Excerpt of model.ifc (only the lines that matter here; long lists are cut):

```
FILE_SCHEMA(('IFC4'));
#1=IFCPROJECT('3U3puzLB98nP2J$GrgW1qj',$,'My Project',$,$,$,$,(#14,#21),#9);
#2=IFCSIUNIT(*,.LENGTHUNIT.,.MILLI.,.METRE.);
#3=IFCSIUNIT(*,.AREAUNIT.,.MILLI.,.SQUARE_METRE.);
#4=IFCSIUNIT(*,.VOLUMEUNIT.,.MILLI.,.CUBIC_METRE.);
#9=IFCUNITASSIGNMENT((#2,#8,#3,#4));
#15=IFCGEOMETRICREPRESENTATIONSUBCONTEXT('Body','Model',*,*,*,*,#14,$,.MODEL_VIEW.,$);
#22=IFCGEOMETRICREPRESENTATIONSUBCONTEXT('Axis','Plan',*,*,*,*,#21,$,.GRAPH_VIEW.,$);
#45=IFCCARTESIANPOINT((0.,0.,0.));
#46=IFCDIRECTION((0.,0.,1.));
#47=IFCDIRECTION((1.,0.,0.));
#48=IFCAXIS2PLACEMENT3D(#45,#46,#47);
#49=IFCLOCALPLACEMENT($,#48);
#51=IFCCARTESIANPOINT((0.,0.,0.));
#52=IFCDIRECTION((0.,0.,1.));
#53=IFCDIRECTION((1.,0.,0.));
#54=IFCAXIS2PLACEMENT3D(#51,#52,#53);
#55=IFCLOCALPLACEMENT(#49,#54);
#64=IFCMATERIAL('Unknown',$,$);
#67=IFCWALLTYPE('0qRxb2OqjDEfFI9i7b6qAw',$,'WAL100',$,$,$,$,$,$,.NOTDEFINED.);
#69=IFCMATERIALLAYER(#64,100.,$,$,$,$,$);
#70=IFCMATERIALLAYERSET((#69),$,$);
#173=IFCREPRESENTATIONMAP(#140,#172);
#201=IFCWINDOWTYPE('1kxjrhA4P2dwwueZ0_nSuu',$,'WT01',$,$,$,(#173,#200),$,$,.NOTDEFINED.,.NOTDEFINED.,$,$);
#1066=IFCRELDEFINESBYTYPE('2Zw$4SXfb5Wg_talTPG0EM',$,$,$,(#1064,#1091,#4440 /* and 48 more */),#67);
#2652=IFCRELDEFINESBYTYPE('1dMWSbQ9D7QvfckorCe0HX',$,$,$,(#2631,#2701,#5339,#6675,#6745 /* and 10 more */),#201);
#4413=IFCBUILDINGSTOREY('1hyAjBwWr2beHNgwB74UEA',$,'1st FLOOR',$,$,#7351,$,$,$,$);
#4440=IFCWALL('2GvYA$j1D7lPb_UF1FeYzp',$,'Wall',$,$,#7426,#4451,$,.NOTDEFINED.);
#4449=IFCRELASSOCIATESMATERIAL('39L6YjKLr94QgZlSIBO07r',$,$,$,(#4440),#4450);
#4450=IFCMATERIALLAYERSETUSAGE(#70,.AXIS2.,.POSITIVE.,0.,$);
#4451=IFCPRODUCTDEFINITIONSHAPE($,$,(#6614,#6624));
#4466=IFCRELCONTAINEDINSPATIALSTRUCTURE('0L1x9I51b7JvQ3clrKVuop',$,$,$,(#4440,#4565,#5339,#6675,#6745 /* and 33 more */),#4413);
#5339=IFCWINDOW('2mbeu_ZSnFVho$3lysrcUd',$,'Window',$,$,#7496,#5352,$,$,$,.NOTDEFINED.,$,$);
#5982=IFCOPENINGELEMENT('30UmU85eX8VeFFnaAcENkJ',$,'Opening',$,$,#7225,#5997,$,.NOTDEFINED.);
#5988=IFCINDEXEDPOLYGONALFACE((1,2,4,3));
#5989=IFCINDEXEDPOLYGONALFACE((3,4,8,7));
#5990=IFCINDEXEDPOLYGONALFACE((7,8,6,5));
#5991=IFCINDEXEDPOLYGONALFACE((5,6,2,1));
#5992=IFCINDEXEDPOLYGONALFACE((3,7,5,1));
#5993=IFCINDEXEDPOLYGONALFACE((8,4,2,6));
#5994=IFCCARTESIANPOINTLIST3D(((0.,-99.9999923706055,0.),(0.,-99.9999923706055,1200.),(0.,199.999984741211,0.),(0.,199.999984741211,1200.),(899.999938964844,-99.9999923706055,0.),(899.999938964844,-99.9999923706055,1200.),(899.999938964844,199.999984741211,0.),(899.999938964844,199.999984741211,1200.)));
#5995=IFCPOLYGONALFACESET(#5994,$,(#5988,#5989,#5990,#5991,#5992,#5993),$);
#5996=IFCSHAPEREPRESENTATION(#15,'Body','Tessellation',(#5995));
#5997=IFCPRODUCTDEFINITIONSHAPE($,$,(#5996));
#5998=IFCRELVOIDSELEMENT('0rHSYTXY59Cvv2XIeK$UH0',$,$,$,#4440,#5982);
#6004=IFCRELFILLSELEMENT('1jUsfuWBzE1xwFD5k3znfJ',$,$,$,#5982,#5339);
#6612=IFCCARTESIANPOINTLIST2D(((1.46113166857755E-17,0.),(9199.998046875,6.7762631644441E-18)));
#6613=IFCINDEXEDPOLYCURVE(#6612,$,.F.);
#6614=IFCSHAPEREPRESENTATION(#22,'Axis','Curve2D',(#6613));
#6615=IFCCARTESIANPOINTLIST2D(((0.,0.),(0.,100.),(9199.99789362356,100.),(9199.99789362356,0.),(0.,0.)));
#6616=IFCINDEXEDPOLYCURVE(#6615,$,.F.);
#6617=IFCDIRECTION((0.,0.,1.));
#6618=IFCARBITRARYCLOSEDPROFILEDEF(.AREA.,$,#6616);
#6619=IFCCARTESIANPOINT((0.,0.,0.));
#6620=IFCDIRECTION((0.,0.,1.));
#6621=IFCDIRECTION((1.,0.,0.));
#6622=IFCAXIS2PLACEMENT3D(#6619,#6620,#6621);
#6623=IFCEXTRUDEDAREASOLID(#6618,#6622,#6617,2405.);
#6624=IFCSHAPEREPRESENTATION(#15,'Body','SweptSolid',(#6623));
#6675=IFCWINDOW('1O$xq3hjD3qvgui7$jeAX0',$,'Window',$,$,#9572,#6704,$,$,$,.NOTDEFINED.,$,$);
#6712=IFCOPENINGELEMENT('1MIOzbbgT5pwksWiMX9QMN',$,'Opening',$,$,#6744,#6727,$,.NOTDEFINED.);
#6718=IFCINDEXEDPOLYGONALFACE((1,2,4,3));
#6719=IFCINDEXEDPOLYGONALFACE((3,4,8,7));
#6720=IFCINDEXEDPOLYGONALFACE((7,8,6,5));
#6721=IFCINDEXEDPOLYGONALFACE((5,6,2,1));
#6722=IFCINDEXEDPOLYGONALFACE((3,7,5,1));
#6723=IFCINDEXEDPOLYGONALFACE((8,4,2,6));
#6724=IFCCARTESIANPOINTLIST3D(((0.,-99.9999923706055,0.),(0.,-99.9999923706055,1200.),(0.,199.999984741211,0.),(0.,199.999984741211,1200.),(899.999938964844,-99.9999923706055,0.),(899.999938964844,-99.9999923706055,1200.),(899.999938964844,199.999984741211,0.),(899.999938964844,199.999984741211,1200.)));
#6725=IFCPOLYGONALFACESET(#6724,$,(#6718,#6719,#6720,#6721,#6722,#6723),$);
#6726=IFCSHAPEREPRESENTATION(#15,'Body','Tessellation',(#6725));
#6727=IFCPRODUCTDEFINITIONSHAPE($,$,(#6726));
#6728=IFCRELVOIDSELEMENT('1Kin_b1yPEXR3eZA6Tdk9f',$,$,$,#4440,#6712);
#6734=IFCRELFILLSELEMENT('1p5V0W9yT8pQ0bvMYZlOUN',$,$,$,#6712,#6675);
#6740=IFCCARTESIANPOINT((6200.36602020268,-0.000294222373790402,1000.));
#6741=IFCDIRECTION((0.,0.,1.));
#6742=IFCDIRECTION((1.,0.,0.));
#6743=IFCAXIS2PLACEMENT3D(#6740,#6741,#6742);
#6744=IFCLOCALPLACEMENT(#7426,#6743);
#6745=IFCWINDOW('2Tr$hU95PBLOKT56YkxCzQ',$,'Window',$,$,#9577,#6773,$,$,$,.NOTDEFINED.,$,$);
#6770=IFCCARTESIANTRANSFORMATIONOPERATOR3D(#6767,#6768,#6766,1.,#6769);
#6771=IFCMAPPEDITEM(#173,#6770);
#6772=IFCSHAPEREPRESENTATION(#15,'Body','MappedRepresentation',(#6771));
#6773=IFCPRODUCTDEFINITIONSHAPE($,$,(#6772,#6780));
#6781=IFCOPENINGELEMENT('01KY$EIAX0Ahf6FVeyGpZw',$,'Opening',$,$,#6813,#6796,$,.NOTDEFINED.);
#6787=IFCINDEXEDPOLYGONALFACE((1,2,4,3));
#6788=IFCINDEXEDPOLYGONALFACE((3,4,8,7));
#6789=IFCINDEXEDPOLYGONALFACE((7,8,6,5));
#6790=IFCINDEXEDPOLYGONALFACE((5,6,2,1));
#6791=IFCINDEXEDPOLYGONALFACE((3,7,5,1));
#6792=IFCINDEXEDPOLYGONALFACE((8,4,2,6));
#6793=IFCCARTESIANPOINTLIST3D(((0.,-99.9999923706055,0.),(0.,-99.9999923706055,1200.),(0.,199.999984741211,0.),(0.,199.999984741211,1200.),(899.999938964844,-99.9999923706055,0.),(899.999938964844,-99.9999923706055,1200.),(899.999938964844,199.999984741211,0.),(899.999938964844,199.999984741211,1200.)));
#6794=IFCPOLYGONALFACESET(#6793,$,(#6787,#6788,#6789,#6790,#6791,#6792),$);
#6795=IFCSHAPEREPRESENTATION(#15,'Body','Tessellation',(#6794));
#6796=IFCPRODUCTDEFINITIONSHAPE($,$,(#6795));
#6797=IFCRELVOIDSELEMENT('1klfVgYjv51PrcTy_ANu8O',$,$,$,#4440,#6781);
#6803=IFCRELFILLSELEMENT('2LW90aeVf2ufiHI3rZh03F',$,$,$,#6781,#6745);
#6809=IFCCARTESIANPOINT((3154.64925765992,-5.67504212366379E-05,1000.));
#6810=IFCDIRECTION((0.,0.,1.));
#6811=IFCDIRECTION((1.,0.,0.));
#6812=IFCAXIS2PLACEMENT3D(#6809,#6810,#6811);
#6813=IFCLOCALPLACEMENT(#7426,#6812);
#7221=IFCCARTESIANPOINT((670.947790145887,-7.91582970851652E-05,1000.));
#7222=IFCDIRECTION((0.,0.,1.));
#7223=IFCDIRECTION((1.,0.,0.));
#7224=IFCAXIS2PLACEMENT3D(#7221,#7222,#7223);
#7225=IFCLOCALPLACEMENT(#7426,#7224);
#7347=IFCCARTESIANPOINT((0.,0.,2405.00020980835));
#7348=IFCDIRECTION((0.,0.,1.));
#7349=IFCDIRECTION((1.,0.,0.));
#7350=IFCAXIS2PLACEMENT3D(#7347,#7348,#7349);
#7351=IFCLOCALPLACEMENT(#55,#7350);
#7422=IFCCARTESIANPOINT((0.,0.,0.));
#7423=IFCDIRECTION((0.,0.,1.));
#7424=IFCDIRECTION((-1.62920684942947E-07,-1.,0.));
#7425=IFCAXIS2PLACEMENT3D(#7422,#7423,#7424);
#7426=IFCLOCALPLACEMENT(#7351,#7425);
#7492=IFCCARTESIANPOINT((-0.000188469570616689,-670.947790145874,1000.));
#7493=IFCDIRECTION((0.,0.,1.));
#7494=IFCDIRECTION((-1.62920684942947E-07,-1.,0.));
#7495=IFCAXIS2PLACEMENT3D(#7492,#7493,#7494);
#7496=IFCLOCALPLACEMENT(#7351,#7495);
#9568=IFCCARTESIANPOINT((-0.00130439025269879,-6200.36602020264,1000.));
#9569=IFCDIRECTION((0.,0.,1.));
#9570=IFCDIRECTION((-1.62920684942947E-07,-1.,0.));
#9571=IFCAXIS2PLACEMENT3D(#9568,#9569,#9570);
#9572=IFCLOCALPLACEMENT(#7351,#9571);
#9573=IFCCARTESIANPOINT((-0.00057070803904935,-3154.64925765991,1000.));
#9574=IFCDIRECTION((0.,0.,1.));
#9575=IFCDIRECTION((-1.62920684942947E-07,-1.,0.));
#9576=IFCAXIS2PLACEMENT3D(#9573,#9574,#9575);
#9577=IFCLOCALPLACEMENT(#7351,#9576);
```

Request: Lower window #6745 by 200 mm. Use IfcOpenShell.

```python
import numpy as np
import ifcopenshell
import ifcopenshell.api.geometry
import ifcopenshell.util.placement
import ifcopenshell.util.unit

model = ifcopenshell.open("model.ifc")
unit_scale = ifcopenshell.util.unit.calculate_unit_scale(model)

window = model.by_guid("2Tr$hU95PBLOKT56YkxCzQ")
opening = window.FillsVoids[0].RelatingOpeningElement
dz = -200.0

shift = np.array([0.0, 0.0, dz])
# The window is not placed relative to its opening, so move both.
for product in (opening, window):
    matrix = ifcopenshell.util.placement.get_local_placement(product.ObjectPlacement)
    matrix[:3, 3] += shift
    ifcopenshell.api.geometry.edit_object_placement(model, product=product, matrix=matrix, is_si=False)

print(f"moved by {dz * unit_scale:+.3f} m")

model.write("model_v2.ifc")
```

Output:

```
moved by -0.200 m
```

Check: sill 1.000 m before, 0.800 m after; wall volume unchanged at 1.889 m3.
